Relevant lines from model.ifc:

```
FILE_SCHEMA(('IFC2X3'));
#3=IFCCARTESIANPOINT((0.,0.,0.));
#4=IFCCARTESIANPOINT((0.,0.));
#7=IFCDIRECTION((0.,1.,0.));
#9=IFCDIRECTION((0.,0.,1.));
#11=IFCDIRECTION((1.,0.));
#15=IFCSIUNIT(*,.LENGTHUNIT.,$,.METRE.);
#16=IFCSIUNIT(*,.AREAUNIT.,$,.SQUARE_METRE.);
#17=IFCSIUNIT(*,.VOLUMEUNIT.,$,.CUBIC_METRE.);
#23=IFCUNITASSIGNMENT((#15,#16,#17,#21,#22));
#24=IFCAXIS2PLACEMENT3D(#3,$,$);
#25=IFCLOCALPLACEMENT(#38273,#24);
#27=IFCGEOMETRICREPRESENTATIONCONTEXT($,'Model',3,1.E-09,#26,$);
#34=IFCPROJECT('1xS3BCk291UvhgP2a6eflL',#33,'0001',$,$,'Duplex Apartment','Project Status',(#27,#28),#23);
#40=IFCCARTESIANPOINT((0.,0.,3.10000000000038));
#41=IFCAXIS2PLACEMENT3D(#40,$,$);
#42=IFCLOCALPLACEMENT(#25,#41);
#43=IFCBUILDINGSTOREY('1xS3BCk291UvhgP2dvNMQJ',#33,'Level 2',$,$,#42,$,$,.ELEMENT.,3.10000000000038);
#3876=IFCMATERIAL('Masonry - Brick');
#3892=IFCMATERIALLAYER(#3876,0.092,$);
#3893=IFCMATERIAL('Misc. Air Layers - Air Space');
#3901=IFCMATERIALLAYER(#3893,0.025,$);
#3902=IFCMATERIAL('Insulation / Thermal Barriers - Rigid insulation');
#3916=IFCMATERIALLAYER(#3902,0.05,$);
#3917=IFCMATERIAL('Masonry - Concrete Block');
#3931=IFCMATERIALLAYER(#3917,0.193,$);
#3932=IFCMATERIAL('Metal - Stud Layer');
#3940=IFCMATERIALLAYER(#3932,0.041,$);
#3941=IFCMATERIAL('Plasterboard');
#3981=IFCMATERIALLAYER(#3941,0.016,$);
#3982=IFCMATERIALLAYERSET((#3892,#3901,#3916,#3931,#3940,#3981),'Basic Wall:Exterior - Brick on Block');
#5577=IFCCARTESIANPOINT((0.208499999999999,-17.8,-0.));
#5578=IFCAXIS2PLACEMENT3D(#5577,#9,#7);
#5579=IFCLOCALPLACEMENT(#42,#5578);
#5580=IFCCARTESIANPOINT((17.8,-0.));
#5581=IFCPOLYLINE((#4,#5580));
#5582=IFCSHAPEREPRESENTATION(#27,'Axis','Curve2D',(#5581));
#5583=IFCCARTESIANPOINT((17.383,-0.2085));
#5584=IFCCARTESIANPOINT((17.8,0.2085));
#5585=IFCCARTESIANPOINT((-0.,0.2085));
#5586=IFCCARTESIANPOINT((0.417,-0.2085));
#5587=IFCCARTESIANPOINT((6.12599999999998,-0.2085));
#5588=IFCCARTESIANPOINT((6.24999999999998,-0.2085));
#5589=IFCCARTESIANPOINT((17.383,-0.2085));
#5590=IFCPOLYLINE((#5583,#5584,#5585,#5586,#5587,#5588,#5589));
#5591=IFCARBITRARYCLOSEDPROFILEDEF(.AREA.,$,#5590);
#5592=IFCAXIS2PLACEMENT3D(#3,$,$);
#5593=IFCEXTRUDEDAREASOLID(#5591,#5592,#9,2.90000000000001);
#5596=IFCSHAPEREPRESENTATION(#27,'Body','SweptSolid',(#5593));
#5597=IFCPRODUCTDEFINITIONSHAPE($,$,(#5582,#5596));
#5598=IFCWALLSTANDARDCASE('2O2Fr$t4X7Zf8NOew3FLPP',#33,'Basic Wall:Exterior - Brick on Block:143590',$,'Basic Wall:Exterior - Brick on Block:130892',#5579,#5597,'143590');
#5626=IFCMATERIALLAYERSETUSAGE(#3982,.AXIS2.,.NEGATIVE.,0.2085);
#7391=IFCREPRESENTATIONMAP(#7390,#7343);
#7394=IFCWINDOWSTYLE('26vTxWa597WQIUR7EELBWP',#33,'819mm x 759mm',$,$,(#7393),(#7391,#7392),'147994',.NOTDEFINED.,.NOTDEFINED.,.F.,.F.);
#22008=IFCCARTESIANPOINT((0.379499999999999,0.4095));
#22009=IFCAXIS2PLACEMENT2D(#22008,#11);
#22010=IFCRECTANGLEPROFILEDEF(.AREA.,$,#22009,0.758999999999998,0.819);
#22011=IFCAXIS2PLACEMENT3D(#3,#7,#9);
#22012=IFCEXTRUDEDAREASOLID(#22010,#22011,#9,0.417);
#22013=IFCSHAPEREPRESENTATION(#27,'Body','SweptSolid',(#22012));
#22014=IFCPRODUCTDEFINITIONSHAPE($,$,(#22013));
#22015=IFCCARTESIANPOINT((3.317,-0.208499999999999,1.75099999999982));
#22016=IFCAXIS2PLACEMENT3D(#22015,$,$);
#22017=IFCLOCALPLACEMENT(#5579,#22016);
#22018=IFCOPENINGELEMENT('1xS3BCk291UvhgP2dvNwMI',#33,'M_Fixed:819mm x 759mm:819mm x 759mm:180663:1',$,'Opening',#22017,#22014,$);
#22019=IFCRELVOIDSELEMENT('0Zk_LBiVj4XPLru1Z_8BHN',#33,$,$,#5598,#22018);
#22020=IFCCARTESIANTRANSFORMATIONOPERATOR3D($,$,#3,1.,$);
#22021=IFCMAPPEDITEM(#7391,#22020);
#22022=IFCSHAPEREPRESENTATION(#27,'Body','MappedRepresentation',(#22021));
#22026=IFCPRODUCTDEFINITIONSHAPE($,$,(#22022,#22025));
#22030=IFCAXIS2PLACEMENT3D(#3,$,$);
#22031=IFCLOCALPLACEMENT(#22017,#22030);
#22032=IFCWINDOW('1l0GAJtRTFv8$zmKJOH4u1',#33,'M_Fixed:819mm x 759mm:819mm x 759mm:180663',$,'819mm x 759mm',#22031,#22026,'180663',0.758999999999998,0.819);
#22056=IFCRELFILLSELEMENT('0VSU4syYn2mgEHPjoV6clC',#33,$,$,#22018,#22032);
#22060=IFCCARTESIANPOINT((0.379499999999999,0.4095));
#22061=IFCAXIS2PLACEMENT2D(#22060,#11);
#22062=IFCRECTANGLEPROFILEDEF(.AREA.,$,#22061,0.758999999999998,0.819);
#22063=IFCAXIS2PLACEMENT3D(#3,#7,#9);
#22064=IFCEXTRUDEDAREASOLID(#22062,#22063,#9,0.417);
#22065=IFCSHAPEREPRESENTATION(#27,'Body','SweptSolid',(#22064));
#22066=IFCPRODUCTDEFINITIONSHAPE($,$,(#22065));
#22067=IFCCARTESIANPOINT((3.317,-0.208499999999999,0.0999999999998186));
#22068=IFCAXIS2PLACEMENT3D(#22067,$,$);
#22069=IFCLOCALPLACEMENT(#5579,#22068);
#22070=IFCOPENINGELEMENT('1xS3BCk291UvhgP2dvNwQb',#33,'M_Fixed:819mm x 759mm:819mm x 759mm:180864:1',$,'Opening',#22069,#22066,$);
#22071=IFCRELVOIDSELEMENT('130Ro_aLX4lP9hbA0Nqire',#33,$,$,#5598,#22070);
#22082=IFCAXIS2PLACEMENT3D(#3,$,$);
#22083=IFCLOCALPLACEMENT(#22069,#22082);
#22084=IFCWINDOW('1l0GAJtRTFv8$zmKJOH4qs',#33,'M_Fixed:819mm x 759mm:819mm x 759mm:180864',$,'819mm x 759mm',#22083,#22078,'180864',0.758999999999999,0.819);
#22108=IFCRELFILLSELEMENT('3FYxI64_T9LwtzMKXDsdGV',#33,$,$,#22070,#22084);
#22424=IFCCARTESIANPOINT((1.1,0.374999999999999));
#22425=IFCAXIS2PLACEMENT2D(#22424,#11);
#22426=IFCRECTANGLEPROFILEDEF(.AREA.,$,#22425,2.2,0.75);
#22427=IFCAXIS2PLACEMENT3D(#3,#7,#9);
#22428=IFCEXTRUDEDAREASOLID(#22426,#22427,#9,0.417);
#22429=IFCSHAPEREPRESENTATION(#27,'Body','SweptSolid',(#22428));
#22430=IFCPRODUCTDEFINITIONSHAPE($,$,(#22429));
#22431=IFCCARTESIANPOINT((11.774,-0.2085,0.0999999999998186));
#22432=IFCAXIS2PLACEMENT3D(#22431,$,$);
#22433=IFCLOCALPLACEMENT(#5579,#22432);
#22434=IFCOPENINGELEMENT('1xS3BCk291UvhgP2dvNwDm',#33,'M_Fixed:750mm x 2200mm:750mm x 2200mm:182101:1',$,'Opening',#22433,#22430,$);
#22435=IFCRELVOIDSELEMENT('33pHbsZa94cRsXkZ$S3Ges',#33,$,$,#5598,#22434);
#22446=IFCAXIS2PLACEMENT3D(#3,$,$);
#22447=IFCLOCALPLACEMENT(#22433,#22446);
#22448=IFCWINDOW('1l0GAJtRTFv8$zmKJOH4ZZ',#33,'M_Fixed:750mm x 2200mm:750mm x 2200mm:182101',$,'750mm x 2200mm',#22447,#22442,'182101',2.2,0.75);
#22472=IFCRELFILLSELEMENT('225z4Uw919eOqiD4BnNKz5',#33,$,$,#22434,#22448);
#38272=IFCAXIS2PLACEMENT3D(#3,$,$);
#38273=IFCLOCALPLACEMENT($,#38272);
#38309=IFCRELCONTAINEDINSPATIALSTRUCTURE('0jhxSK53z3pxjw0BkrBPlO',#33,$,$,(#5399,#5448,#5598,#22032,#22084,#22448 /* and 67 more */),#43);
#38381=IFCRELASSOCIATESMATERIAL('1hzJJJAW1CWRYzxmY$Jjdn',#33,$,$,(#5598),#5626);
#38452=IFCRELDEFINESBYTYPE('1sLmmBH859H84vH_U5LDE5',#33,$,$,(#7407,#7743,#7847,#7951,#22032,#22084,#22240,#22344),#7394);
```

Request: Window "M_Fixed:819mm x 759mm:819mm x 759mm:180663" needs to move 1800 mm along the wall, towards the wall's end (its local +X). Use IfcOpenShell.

```python
import ifcopenshell
import ifcopenshell.api.geometry
import ifcopenshell.util.placement
import ifcopenshell.util.unit

model = ifcopenshell.open("model.ifc")
unit_scale = ifcopenshell.util.unit.calculate_unit_scale(model)

window = model.by_guid("1l0GAJtRTFv8$zmKJOH4u1")
opening = window.FillsVoids[0].RelatingOpeningElement
wall = opening.VoidsElements[0].RelatingBuildingElement

wall_matrix = ifcopenshell.util.placement.get_local_placement(wall.ObjectPlacement)
shift = wall_matrix[:3, 0] * 1.8 / unit_scale
before = ifcopenshell.util.placement.get_local_placement(window.ObjectPlacement)[:3, 3].copy()

# The window is placed relative to its opening, so it follows when the opening moves.
matrix = ifcopenshell.util.placement.get_local_placement(opening.ObjectPlacement)
matrix[:3, 3] += shift
ifcopenshell.api.geometry.edit_object_placement(
    model, product=opening, matrix=matrix, is_si=False, should_transform_children=True
)

after = ifcopenshell.util.placement.get_local_placement(window.ObjectPlacement)[:3, 3]
print("window moved by", (after - before).round(3) + 0.0)

model.write("model_rev.ifc")
```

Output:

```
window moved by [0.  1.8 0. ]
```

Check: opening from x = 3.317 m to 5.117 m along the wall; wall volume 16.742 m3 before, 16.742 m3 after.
